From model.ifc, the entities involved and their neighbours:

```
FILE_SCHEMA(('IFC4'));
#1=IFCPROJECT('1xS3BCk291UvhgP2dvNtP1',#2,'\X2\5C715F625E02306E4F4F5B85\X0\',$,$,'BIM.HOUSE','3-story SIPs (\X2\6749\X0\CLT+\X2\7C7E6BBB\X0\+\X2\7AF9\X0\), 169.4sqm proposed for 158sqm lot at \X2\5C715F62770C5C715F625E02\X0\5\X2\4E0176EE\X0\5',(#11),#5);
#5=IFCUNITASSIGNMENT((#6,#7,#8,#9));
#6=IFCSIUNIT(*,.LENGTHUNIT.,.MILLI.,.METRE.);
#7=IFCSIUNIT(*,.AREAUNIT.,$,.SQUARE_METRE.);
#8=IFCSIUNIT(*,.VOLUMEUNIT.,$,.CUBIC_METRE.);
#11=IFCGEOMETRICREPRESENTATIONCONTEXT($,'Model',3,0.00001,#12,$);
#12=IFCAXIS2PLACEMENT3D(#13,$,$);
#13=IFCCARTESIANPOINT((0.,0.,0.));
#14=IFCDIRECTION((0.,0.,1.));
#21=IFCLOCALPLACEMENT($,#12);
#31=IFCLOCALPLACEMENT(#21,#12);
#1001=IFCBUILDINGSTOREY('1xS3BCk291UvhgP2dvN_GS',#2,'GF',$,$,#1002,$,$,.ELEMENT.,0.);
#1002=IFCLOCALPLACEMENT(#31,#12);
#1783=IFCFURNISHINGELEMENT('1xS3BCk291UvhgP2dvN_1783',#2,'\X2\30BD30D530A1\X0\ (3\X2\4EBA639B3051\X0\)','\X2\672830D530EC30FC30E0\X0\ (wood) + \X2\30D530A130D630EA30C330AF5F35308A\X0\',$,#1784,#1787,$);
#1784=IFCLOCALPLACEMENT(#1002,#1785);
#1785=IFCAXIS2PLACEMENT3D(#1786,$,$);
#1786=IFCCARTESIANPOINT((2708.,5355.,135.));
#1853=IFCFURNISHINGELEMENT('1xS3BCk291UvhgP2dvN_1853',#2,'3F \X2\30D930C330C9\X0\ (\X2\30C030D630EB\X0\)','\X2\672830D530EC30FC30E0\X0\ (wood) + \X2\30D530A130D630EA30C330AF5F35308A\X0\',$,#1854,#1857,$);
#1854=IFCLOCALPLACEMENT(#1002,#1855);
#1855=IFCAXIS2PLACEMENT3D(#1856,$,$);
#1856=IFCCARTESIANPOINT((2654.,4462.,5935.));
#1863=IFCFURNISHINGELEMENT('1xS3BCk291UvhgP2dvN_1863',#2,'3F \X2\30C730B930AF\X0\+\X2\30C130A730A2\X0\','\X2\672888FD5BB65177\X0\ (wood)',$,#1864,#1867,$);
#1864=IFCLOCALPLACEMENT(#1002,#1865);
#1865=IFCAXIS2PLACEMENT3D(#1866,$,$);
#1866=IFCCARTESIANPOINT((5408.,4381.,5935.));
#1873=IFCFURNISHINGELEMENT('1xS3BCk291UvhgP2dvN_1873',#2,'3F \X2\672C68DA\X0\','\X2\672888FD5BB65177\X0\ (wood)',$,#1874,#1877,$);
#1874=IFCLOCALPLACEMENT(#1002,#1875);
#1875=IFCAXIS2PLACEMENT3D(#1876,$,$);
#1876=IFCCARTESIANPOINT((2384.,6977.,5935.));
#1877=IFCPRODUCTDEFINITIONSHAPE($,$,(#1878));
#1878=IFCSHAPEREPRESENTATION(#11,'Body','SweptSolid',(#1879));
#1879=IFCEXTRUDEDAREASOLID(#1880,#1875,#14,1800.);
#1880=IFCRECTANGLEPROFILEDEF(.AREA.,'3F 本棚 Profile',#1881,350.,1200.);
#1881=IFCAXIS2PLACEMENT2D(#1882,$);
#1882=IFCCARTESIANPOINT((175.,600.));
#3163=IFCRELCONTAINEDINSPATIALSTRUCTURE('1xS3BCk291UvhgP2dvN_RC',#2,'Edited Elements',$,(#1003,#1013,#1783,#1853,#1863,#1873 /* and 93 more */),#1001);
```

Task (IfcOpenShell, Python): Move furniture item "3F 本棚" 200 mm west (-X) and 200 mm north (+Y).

```python
import ifcopenshell
import ifcopenshell.api.geometry
import ifcopenshell.util.placement
import ifcopenshell.util.unit

model = ifcopenshell.open("model.ifc")
unit_scale = ifcopenshell.util.unit.calculate_unit_scale(model)

item = model.by_guid("1xS3BCk291UvhgP2dvN_1873")
matrix = ifcopenshell.util.placement.get_local_placement(item.ObjectPlacement)
matrix[0, 3] -= 0.2 / unit_scale
matrix[1, 3] += 0.2 / unit_scale
ifcopenshell.api.geometry.edit_object_placement(model, product=item, matrix=matrix, is_si=False)

print(ifcopenshell.util.placement.get_local_placement(item.ObjectPlacement).round(3) + 0.0)

model.write("model_edited.ifc")
```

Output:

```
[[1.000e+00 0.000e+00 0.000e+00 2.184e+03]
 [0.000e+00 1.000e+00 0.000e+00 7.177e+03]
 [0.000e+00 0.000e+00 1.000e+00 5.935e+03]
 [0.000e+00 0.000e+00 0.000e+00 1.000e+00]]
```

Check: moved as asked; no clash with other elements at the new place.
